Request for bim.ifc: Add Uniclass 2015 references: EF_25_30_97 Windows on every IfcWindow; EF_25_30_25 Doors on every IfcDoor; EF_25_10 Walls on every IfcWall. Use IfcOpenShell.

First a look at what the model holds.

```python
import ifcopenshell

model = ifcopenshell.open("bim.ifc")
print(model.schema)
print("classifications:", [c.Name for c in model.by_type("IfcClassification")])
for ifc_class in ("IfcDoor", "IfcRoof", "IfcStair", "IfcWall", "IfcWindow"):
    print(ifc_class, len(model.by_type(ifc_class)))
```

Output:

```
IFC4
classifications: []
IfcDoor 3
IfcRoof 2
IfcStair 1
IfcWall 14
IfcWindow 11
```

```python
import ifcopenshell
import ifcopenshell.api.classification

model = ifcopenshell.open("bim.ifc")

system = ifcopenshell.api.classification.add_classification(model, classification="Uniclass 2015")

codes = {
    "IfcWindow": ("EF_25_30_97", "Windows"),
    "IfcDoor": ("EF_25_30_25", "Doors"),
    "IfcWall": ("EF_25_10", "Walls"),
}
for ifc_class, (code, name) in codes.items():
    products = model.by_type(ifc_class)
    ifcopenshell.api.classification.add_reference(
        model, products=products, classification=system, identification=code, name=name
    )
    print(code, len(products))

model.write("bim_rev.ifc")
```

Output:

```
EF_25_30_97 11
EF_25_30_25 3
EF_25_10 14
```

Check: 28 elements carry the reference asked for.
